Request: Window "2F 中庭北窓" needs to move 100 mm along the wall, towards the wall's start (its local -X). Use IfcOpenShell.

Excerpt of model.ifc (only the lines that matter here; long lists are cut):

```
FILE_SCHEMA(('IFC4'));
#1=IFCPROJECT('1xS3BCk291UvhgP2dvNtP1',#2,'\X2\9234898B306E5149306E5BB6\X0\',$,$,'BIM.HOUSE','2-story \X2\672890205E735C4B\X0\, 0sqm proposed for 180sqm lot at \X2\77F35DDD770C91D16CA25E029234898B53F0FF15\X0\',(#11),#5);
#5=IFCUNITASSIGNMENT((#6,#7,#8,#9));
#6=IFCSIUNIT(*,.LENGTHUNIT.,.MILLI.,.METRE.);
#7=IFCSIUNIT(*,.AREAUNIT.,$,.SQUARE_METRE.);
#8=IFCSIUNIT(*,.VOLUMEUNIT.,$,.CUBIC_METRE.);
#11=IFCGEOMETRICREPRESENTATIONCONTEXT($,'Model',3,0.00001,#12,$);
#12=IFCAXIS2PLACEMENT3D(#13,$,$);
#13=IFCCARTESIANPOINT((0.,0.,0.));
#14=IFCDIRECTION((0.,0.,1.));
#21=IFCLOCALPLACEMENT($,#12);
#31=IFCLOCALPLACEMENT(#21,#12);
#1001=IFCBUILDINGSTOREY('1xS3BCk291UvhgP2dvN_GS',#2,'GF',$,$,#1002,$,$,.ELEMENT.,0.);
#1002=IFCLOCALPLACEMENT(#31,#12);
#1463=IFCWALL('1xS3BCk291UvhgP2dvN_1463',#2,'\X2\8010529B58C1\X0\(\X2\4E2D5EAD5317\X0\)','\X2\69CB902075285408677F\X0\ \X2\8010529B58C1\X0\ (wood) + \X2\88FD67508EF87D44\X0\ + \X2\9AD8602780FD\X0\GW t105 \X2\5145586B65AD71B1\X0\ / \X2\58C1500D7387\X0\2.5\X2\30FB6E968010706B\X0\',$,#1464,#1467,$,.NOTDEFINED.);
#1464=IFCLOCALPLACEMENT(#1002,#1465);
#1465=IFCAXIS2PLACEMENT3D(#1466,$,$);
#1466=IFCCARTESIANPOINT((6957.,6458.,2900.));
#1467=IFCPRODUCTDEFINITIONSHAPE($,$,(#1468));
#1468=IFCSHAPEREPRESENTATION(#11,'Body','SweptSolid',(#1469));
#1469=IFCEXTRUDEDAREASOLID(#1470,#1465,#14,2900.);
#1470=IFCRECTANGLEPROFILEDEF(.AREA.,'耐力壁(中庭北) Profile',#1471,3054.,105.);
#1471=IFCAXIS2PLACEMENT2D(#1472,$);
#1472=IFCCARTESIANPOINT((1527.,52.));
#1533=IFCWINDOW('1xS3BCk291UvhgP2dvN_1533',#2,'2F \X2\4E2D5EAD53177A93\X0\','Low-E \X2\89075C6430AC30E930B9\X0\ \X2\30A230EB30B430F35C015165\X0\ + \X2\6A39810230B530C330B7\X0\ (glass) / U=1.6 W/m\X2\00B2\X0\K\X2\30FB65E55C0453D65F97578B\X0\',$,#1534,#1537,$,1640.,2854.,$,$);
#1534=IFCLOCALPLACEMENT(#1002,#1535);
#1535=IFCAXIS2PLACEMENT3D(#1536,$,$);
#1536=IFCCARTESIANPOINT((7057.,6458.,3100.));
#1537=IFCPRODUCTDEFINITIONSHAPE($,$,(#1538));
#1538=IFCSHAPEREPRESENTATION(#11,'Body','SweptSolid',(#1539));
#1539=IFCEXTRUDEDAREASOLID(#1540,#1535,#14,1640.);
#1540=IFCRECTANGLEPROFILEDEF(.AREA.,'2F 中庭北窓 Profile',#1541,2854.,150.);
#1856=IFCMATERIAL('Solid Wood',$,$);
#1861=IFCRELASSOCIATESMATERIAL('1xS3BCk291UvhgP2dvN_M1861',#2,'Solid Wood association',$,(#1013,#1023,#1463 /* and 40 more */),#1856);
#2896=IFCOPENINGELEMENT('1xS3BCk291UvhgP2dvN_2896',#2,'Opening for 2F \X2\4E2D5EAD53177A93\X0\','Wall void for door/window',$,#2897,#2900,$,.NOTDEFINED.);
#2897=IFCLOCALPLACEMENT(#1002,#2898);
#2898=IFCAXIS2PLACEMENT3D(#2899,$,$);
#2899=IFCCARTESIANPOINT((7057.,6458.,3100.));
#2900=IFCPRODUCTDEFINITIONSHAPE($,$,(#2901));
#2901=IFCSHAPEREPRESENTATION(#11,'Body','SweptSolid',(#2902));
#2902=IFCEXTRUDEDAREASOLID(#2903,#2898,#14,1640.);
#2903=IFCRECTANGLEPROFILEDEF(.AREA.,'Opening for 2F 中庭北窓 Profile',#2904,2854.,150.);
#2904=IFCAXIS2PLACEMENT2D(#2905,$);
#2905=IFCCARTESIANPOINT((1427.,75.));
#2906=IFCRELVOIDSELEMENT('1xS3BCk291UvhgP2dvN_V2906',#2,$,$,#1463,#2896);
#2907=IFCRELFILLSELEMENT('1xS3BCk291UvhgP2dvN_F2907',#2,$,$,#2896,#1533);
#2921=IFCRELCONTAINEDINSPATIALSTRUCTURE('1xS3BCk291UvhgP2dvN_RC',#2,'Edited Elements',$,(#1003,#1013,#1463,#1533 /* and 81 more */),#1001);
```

```python
import ifcopenshell
import ifcopenshell.api.geometry
import ifcopenshell.util.placement
import ifcopenshell.util.unit

model = ifcopenshell.open("model.ifc")
unit_scale = ifcopenshell.util.unit.calculate_unit_scale(model)

window = model.by_guid("1xS3BCk291UvhgP2dvN_1533")
opening = window.FillsVoids[0].RelatingOpeningElement
wall = opening.VoidsElements[0].RelatingBuildingElement

wall_matrix = ifcopenshell.util.placement.get_local_placement(wall.ObjectPlacement)
shift = wall_matrix[:3, 0] * -0.1 / unit_scale
before = ifcopenshell.util.placement.get_local_placement(window.ObjectPlacement)[:3, 3].copy()

# The window is not placed relative to its opening, so move both.
for product in (opening, window):
    matrix = ifcopenshell.util.placement.get_local_placement(product.ObjectPlacement)
    matrix[:3, 3] += shift
    ifcopenshell.api.geometry.edit_object_placement(model, product=product, matrix=matrix, is_si=False)

after = ifcopenshell.util.placement.get_local_placement(window.ObjectPlacement)[:3, 3]
print("window moved by", (after - before).round(3) + 0.0)

model.write("model_rev.ifc")
```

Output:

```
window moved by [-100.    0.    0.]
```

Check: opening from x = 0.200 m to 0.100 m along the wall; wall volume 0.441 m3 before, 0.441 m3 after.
